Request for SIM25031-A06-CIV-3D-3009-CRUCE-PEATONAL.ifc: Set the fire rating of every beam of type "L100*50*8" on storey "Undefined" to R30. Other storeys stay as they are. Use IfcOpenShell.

First a look at what the model holds.

```python
import ifcopenshell
import ifcopenshell.util.element

model = ifcopenshell.open("SIM25031-A06-CIV-3D-3009-CRUCE-PEATONAL.ifc")
print(model.schema)
storey = next(s for s in model.by_type("IfcBuildingStorey") if s.Name == "Undefined")
beams = [e for e in ifcopenshell.util.element.get_decomposition(storey) if e.is_a("IfcBeam")]
seen = {}
for e in beams:
    element_type = ifcopenshell.util.element.get_type(e)
    key = (element_type.Name if element_type != e and element_type else None, ifcopenshell.util.element.get_pset(e, "Pset_BeamCommon", "FireRating"))
    seen[key] = seen.get(key, 0) + 1
for (name, value), count in sorted(seen.items(), key=str):
    print(count, "x", name, "|", value)
```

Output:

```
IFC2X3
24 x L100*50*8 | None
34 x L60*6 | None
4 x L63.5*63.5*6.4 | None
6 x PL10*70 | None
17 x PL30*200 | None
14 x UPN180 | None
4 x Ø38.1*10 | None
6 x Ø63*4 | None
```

```python
import ifcopenshell
import ifcopenshell.api.pset
import ifcopenshell.util.element

model = ifcopenshell.open("SIM25031-A06-CIV-3D-3009-CRUCE-PEATONAL.ifc")

storey = next(s for s in model.by_type("IfcBuildingStorey") if s.Name == "Undefined")
beams = [e for e in ifcopenshell.util.element.get_decomposition(storey) if e.is_a("IfcBeam")]

count = 0
for e in beams:
    element_type = ifcopenshell.util.element.get_type(e)
    if element_type in (None, e) or element_type.Name != "L100*50*8":
        continue
    found = ifcopenshell.util.element.get_pset(e, "Pset_BeamCommon", should_inherit=False)
    if found:
        pset = model.by_id(found["id"])
        if len(ifcopenshell.util.element.get_elements_by_pset(pset)) > 1:
            pset = ifcopenshell.api.pset.unshare_pset(model, products=[e], pset=pset)[0]
    else:
        pset = ifcopenshell.api.pset.add_pset(model, product=e, name="Pset_BeamCommon")
    ifcopenshell.api.pset.edit_pset(model, pset=pset, properties={"FireRating": "R30"})
    count += 1

print(count, "beams updated")

model.write("SIM25031-A06-CIV-3D-3009-CRUCE-PEATONAL_v2.ifc")
```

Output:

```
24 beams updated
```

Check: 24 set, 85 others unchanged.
